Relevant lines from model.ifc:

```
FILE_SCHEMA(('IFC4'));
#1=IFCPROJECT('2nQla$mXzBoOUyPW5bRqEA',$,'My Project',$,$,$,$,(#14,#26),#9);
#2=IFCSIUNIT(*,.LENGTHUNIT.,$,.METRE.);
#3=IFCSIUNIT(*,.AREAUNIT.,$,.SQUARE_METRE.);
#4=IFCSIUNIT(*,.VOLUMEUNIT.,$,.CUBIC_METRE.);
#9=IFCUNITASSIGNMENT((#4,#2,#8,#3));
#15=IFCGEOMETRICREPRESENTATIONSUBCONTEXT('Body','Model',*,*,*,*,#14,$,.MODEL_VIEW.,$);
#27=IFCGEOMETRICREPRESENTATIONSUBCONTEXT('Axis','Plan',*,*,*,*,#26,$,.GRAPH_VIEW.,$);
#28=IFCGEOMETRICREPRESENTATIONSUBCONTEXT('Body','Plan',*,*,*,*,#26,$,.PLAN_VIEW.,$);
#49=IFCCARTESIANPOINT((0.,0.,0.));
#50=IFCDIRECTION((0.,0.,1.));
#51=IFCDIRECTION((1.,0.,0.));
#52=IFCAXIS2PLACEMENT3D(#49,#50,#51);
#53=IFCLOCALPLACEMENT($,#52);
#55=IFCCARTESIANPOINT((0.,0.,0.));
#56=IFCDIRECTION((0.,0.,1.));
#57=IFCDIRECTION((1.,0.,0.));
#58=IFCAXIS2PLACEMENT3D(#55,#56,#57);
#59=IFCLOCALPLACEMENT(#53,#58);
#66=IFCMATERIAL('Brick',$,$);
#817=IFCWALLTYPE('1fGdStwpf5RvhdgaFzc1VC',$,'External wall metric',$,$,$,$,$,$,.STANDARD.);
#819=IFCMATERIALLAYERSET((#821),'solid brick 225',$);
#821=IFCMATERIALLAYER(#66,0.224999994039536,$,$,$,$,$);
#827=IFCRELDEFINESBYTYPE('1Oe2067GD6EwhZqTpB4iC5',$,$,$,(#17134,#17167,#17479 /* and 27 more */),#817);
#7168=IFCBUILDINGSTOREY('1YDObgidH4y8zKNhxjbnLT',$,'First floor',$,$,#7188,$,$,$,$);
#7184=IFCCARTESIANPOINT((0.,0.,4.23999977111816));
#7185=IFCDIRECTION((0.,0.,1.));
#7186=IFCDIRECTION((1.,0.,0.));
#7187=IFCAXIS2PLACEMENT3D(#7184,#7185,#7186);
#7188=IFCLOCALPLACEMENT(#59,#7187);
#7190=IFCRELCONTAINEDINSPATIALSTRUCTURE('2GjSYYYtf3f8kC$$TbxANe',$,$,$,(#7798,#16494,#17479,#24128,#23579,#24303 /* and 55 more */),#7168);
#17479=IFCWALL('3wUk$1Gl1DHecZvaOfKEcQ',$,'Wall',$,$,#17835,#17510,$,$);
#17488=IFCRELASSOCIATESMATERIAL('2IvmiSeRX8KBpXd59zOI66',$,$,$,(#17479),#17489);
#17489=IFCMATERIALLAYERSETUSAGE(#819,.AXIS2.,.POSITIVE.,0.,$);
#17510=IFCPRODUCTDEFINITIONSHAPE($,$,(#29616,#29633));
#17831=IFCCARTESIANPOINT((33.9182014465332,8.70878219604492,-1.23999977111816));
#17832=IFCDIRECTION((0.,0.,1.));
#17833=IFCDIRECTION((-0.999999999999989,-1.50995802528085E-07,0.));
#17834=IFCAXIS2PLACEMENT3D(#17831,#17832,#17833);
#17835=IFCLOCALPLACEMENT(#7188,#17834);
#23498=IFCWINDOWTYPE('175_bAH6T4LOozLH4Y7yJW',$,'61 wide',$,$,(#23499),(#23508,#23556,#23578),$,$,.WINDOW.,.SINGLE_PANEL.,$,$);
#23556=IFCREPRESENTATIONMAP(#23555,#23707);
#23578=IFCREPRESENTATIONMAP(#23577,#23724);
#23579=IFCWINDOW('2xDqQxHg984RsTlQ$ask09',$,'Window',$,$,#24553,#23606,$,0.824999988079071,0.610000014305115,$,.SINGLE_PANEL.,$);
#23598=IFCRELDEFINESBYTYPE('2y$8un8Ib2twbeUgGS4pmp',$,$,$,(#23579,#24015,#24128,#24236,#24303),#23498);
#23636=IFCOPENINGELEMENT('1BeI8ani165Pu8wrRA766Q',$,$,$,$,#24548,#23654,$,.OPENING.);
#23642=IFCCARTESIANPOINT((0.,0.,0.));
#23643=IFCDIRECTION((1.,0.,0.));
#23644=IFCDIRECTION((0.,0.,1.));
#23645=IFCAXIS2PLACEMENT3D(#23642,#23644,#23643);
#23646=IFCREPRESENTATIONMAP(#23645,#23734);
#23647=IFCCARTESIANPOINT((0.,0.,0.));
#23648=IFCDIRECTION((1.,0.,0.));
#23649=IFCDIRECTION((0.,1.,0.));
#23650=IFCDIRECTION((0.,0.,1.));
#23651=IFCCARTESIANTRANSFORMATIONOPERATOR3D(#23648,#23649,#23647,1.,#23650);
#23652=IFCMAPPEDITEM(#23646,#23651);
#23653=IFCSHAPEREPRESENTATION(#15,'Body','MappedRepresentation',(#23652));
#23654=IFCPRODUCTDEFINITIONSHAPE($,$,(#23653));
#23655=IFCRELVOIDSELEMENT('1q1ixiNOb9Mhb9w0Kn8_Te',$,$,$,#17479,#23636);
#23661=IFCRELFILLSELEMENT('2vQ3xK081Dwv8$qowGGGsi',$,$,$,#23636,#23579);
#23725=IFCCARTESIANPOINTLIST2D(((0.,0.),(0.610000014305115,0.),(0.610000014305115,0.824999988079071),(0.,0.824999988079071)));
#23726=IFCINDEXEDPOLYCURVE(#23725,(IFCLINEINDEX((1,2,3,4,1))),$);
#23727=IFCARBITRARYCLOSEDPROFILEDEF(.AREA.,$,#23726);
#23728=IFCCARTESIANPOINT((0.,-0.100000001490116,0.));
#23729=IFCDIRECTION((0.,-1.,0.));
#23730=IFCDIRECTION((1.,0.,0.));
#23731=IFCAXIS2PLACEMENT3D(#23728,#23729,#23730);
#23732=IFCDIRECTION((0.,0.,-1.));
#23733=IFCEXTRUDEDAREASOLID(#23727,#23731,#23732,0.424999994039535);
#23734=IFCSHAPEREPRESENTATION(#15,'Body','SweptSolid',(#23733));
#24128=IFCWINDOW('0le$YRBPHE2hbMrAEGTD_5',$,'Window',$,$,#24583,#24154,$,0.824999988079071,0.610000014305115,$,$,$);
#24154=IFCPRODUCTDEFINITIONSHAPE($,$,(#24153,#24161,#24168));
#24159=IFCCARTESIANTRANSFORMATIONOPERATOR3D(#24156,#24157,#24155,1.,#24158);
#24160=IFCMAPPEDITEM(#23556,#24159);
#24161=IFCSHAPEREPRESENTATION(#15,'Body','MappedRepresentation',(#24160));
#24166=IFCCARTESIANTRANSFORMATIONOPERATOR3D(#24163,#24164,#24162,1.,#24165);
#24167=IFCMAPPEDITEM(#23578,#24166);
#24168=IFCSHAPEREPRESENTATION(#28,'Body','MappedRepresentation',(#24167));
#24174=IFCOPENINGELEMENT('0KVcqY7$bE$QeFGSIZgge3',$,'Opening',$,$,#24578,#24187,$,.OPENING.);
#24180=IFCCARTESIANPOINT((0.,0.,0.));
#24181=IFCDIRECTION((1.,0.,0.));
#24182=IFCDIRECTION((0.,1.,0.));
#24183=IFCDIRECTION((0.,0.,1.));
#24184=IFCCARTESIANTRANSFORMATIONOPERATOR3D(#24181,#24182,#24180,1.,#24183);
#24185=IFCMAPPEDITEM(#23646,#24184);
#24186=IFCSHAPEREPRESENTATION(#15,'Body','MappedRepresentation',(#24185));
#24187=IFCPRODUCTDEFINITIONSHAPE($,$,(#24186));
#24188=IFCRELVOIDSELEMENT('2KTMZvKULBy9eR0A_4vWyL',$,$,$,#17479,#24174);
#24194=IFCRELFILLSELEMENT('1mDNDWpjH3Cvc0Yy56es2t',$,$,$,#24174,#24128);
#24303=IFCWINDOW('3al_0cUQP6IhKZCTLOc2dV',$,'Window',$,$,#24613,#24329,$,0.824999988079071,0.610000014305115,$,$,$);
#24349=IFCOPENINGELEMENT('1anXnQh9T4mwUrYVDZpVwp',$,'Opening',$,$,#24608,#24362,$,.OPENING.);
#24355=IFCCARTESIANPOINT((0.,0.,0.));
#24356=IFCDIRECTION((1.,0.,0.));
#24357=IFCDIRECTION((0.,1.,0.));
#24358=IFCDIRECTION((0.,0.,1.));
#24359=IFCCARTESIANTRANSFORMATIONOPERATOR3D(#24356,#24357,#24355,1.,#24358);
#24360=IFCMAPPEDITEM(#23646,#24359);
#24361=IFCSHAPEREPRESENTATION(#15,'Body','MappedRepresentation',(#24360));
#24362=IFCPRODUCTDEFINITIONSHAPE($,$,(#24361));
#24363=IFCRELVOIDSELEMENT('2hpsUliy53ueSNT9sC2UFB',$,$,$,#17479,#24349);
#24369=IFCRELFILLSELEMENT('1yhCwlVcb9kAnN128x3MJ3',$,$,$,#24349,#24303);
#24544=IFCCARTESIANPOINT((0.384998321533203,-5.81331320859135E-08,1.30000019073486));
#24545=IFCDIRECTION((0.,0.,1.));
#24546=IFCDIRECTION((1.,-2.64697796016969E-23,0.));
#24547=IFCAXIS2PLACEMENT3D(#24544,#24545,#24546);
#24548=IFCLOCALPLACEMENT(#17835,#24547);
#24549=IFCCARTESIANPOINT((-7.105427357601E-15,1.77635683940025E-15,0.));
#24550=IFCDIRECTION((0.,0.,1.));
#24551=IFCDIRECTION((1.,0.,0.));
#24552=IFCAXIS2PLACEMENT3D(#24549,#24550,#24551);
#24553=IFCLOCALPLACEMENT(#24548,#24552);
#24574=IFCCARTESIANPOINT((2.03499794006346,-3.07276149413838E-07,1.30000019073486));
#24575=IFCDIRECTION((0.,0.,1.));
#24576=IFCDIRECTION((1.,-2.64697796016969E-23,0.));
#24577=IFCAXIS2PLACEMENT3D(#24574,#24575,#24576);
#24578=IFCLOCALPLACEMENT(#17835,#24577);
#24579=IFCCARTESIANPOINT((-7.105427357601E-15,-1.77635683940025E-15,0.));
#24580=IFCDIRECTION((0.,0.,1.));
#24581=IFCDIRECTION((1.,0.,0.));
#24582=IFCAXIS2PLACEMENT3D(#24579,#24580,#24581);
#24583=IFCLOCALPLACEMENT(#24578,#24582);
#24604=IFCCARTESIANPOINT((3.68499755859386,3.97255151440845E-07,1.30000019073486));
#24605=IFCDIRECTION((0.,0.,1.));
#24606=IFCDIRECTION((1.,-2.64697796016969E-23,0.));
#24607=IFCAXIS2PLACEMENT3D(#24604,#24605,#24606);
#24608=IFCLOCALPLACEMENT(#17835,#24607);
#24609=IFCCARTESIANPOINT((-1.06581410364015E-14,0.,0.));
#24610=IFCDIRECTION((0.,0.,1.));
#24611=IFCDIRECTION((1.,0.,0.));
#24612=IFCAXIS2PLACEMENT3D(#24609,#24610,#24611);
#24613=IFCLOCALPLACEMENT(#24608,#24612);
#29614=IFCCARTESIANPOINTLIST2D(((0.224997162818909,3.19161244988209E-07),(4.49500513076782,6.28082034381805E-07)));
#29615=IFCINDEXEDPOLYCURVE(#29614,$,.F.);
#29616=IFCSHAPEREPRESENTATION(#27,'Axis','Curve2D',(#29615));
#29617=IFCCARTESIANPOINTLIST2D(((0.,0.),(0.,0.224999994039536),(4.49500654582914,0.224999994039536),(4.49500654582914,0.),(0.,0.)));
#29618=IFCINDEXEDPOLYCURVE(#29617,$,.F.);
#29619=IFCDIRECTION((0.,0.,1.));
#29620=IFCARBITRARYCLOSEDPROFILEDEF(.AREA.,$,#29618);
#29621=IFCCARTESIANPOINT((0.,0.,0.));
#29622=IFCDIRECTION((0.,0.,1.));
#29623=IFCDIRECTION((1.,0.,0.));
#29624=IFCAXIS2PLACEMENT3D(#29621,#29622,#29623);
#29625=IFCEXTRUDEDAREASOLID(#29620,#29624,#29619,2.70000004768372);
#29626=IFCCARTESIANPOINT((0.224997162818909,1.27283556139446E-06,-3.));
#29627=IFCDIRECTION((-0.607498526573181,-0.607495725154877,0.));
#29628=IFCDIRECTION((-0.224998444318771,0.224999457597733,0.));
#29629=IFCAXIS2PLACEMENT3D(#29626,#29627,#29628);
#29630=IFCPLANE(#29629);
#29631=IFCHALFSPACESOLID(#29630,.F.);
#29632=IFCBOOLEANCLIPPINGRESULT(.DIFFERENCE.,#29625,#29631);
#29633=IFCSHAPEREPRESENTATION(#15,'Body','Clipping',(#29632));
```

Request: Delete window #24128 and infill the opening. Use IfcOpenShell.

```python
import ifcopenshell
import ifcopenshell.api.feature
import ifcopenshell.api.root
import ifcopenshell.geom
import ifcopenshell.util.shape

model = ifcopenshell.open("model.ifc")
settings = ifcopenshell.geom.settings()


def volume(element):
    """Net volume in cubic metres, openings subtracted."""
    shape = ifcopenshell.geom.create_shape(settings, element)
    return ifcopenshell.util.shape.get_volume(shape.geometry)


window = model.by_id(24128)
opening = window.FillsVoids[0].RelatingOpeningElement
wall = opening.VoidsElements[0].RelatingBuildingElement
before = volume(wall)

ifcopenshell.api.root.remove_product(model, product=window)
ifcopenshell.api.feature.remove_feature(model, feature=opening)

after = volume(wall)

print(f"wall volume {before:.3f} -> {after:.3f} m3")

model.write("model_edited.ifc")
```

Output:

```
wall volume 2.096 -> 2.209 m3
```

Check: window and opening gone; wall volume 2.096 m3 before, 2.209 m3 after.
